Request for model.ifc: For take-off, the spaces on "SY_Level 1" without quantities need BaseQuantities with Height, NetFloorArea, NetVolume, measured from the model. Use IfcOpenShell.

First a look at what the model holds.

```python
import ifcopenshell
import ifcopenshell.util.element
import ifcopenshell.util.unit

model = ifcopenshell.open("model.ifc")
print(model.schema)
for unit_type in ("LENGTHUNIT", "AREAUNIT", "VOLUMEUNIT"):
    print(unit_type, ifcopenshell.util.unit.calculate_unit_scale(model, unit_type))
storey = next(s for s in model.by_type("IfcBuildingStorey") if s.Name == "SY_Level 1")
spaces = [e for e in ifcopenshell.util.element.get_decomposition(storey) if e.is_a("IfcSpace")]
for e in sorted(spaces, key=lambda e: e.id()):
    print(e.id(), e.is_a(), e.Name, list(ifcopenshell.util.element.get_psets(e, qtos_only=True)), sep=" | ")
```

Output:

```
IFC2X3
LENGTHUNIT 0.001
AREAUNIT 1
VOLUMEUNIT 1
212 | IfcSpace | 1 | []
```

```python
import ifcopenshell
import ifcopenshell.api.pset
import ifcopenshell.geom
import ifcopenshell.util.element
import ifcopenshell.util.shape
import ifcopenshell.util.unit

model = ifcopenshell.open("model.ifc")
unit_scale = ifcopenshell.util.unit.calculate_unit_scale(model)
area_scale = ifcopenshell.util.unit.calculate_unit_scale(model, "AREAUNIT")
volume_scale = ifcopenshell.util.unit.calculate_unit_scale(model, "VOLUMEUNIT")
settings = ifcopenshell.geom.settings()

storey = next(s for s in model.by_type("IfcBuildingStorey") if s.Name == "SY_Level 1")
spaces = [e for e in ifcopenshell.util.element.get_decomposition(storey) if e.is_a("IfcSpace")]

for e in sorted(spaces, key=lambda e: e.id()):
    if ifcopenshell.util.element.get_psets(e, qtos_only=True, should_inherit=False):
        continue
    # Geometry comes back in metres, in the element's own axes.
    shape = ifcopenshell.geom.create_shape(settings, e)
    values = {
        "Height": ifcopenshell.util.shape.get_z(shape.geometry) / unit_scale,
        "NetFloorArea": ifcopenshell.util.shape.get_footprint_area(shape.geometry) / area_scale,
        "NetVolume": ifcopenshell.util.shape.get_volume(shape.geometry) / volume_scale,
    }
    qto = ifcopenshell.api.pset.add_qto(model, product=e, name="BaseQuantities")
    ifcopenshell.api.pset.edit_qto(model, qto=qto, properties=values)
    print(e.id(), {k: round(v, 3) for k, v in values.items()})

model.write("model_updated.ifc")
```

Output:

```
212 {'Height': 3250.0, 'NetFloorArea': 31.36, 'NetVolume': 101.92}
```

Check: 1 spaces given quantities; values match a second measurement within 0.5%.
